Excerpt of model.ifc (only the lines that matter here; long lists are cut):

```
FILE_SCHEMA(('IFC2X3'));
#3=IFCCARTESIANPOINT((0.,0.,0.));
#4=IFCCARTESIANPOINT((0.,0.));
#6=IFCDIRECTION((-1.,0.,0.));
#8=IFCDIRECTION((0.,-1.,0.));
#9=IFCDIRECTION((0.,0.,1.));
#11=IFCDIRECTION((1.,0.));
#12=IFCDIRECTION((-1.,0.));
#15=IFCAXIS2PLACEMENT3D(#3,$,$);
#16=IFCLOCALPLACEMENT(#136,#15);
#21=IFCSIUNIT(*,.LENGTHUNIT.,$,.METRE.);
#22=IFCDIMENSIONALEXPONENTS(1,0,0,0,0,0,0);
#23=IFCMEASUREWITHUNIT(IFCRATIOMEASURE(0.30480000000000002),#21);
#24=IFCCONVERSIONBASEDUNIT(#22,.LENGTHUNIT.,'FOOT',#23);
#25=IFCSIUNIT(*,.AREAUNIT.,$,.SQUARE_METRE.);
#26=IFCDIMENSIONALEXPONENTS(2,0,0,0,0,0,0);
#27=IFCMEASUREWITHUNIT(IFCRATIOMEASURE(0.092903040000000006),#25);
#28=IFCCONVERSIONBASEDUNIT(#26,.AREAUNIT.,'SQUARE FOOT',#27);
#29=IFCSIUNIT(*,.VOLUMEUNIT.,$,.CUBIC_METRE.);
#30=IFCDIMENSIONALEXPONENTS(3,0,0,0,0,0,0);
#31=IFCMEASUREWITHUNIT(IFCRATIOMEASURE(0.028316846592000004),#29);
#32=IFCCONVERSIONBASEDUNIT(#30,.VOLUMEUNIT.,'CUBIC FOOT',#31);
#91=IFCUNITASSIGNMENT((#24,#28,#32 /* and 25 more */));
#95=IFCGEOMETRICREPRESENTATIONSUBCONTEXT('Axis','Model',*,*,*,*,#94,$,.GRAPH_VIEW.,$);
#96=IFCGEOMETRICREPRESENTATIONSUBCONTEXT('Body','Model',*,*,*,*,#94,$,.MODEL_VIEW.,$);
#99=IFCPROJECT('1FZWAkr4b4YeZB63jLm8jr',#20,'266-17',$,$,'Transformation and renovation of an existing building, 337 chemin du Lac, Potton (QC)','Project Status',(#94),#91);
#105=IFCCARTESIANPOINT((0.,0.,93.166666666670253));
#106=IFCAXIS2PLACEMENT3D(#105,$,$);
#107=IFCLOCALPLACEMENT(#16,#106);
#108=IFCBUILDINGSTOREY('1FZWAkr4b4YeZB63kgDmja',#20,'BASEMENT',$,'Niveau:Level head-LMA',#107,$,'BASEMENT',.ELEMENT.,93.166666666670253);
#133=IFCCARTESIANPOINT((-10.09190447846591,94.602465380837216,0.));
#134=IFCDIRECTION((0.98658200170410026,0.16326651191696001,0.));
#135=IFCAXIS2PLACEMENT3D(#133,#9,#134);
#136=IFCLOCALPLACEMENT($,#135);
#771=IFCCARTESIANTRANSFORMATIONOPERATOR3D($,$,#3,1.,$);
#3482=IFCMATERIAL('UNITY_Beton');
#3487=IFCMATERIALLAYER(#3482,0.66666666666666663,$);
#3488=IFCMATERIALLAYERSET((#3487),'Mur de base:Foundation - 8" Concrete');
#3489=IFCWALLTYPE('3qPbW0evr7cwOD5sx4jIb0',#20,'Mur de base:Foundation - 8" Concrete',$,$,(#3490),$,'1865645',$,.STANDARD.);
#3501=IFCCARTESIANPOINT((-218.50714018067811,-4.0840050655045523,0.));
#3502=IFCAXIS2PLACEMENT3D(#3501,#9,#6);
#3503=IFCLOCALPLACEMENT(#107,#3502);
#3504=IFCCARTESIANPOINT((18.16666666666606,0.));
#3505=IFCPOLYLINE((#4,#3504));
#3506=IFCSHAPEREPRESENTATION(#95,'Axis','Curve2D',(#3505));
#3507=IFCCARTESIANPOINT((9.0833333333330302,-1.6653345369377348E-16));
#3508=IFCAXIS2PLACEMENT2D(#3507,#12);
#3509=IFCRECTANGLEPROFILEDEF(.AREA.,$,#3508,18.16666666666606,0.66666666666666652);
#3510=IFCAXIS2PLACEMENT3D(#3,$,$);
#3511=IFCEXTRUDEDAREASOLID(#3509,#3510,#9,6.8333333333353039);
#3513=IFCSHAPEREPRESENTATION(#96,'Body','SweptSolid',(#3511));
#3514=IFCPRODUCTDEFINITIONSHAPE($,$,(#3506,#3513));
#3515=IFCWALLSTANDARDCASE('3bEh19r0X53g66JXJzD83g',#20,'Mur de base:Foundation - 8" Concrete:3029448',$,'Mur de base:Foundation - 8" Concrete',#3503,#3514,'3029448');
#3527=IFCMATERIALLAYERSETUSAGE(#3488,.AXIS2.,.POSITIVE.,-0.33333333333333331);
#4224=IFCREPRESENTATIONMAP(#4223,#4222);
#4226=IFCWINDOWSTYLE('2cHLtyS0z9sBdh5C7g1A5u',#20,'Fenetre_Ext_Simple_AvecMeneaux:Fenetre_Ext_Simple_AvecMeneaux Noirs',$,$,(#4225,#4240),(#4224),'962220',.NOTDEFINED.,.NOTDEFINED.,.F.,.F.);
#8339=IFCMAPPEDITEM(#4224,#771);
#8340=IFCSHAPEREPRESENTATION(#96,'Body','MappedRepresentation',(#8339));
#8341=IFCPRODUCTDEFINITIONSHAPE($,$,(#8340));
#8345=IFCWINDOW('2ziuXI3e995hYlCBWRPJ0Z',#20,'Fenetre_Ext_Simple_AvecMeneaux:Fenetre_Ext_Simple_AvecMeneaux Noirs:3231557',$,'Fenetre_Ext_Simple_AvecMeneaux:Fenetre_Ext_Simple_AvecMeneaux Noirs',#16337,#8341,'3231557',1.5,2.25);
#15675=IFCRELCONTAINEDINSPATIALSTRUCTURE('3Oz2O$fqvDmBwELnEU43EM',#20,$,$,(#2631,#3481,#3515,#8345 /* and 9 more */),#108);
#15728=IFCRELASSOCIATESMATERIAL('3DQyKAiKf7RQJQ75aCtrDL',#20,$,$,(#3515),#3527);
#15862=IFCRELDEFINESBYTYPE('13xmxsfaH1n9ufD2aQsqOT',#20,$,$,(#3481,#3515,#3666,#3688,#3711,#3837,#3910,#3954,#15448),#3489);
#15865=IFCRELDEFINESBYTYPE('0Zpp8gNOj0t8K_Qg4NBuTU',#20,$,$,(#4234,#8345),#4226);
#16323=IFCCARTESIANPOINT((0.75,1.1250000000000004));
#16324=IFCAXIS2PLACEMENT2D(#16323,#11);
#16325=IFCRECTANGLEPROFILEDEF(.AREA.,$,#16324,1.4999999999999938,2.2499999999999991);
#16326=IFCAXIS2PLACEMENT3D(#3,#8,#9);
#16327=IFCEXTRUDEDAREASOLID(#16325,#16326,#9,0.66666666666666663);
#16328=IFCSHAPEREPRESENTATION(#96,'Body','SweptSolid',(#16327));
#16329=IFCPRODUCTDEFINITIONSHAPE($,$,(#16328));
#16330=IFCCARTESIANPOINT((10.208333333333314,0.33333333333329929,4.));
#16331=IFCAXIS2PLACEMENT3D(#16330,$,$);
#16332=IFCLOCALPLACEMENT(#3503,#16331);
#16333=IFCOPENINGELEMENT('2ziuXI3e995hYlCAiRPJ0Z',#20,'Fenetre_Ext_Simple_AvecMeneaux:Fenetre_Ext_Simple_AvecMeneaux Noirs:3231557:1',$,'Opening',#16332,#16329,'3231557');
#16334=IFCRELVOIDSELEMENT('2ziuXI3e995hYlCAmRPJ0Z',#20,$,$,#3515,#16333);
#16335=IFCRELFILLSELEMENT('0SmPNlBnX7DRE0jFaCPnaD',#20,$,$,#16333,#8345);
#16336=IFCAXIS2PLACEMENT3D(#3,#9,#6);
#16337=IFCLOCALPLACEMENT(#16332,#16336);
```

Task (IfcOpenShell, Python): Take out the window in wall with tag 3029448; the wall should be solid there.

```python
import ifcopenshell
import ifcopenshell.api.feature
import ifcopenshell.api.root
import ifcopenshell.geom
import ifcopenshell.util.shape

model = ifcopenshell.open("model.ifc")
settings = ifcopenshell.geom.settings()


def volume(element):
    """Net volume in cubic metres, openings subtracted."""
    shape = ifcopenshell.geom.create_shape(settings, element)
    return ifcopenshell.util.shape.get_volume(shape.geometry)


window = model.by_guid("2ziuXI3e995hYlCBWRPJ0Z")
opening = window.FillsVoids[0].RelatingOpeningElement
wall = opening.VoidsElements[0].RelatingBuildingElement
before = volume(wall)

ifcopenshell.api.root.remove_product(model, product=window)
ifcopenshell.api.feature.remove_feature(model, feature=opening)

after = volume(wall)

print(f"wall volume {before:.3f} -> {after:.3f} m3")

model.write("model_rev.ifc")
```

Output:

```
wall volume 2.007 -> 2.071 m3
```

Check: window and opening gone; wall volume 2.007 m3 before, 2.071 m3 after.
